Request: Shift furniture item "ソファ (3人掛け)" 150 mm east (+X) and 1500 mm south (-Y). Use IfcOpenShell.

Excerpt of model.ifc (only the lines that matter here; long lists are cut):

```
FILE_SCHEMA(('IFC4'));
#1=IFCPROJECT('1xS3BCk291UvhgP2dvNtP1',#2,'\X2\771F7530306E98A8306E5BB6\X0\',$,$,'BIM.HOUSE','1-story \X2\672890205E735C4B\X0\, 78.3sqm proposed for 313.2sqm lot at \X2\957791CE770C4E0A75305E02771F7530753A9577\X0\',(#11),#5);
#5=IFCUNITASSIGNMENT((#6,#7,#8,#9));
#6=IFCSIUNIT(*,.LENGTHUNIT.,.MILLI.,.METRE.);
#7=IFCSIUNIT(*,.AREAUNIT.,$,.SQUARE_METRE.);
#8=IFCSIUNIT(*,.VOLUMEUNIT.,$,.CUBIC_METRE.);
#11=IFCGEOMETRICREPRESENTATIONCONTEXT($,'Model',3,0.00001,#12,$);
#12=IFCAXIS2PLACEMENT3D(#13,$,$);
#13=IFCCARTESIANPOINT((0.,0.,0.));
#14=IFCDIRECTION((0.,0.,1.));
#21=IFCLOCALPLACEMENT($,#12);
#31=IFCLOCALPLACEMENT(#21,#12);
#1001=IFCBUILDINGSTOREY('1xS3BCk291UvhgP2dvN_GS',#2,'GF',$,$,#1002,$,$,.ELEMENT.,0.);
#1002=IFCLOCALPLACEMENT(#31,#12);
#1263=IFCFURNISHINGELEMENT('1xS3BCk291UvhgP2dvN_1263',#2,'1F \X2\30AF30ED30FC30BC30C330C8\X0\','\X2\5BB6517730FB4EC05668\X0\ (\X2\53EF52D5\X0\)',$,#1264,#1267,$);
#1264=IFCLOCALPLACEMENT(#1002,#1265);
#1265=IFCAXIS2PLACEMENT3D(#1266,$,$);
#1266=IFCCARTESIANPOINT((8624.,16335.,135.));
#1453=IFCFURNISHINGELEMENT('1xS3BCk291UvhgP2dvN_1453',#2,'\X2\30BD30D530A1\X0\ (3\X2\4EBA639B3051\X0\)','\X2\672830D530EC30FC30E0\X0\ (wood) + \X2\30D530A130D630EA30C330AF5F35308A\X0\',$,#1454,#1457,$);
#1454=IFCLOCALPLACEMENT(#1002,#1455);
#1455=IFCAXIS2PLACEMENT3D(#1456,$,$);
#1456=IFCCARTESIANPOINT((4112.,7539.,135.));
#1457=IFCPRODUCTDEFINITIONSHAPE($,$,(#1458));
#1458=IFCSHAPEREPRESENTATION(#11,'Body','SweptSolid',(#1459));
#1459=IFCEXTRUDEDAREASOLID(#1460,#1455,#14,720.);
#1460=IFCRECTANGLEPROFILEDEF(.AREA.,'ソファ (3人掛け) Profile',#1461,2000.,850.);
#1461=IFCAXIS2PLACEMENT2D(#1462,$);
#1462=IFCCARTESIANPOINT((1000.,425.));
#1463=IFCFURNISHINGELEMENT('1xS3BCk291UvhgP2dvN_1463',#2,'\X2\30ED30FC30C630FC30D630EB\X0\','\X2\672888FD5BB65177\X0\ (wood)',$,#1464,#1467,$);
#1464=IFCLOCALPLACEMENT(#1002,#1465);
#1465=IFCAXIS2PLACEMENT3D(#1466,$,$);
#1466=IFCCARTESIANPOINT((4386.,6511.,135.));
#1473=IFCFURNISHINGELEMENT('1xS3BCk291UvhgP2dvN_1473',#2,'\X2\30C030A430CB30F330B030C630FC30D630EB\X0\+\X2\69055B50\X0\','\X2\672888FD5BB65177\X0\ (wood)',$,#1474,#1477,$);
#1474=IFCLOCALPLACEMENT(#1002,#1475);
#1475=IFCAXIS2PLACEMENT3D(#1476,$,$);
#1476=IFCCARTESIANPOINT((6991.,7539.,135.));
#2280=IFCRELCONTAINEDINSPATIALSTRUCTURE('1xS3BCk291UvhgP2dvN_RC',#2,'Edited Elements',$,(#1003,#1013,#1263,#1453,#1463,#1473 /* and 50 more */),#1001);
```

```python
import ifcopenshell
import ifcopenshell.api.geometry
import ifcopenshell.util.placement

model = ifcopenshell.open("model.ifc")

item = model.by_guid("1xS3BCk291UvhgP2dvN_1453")
matrix = ifcopenshell.util.placement.get_local_placement(item.ObjectPlacement)
matrix[0, 3] += 150.0
matrix[1, 3] -= 1500.0
ifcopenshell.api.geometry.edit_object_placement(model, product=item, matrix=matrix, is_si=False)

print(ifcopenshell.util.placement.get_local_placement(item.ObjectPlacement).round(3) + 0.0)

model.write("model_edited.ifc")
```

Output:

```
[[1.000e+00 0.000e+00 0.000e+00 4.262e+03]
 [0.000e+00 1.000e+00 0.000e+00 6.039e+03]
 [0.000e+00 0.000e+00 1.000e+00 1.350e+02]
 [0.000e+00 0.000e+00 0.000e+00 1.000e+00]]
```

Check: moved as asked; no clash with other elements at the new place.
